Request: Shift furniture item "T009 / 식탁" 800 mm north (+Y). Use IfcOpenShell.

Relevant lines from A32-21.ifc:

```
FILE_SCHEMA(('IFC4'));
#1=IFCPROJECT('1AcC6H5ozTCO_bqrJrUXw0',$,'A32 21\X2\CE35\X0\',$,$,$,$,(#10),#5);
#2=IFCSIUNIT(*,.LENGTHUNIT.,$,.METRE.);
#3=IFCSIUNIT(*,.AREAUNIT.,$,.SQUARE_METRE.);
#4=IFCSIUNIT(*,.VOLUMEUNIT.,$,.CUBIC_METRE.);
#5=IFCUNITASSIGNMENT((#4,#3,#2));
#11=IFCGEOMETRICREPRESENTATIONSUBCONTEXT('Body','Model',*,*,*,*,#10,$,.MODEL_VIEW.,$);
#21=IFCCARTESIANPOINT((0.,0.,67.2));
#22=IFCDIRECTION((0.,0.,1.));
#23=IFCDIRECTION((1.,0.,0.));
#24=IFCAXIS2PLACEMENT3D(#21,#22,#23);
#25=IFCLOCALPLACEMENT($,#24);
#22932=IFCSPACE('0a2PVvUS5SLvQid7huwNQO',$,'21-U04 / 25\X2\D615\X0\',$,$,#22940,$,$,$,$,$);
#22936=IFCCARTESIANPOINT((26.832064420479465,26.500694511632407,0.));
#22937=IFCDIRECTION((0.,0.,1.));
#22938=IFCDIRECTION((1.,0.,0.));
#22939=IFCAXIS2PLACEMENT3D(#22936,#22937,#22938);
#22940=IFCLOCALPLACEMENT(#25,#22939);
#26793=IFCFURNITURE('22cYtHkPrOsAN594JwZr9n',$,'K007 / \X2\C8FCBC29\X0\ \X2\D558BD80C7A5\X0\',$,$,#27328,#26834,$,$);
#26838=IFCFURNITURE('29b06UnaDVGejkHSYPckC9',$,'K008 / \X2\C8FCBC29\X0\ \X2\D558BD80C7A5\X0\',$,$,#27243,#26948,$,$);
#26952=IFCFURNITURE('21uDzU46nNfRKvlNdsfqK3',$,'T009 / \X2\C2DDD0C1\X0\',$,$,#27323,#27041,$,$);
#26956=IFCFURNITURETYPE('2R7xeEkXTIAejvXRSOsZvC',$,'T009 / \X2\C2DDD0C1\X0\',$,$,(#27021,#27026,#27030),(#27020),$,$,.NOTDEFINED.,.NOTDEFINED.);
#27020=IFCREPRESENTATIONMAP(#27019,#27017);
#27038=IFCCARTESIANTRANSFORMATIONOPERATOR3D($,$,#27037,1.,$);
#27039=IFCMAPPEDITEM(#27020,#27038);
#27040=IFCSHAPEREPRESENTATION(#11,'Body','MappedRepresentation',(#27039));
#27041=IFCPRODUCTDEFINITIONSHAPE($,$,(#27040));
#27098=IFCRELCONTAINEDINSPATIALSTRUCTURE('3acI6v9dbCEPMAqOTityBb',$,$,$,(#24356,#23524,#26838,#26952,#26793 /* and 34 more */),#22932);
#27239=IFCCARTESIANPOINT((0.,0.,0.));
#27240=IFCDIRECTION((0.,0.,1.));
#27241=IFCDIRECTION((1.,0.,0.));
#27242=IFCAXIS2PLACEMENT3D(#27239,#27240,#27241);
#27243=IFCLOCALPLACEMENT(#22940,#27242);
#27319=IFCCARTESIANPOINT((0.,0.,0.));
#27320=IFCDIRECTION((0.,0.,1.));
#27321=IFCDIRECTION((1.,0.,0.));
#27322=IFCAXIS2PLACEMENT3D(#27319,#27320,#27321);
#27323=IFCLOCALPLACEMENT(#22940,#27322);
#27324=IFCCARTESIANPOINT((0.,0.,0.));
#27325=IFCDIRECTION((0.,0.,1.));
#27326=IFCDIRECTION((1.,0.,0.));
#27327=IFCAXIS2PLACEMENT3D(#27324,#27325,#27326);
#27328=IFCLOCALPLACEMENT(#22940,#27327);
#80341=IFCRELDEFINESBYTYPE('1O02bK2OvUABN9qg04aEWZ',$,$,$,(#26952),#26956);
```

```python
import ifcopenshell
import ifcopenshell.api.geometry
import ifcopenshell.util.placement

model = ifcopenshell.open("A32-21.ifc")

item = model.by_id(26952)
matrix = ifcopenshell.util.placement.get_local_placement(item.ObjectPlacement)
matrix[1, 3] += 0.8
ifcopenshell.api.geometry.edit_object_placement(model, product=item, matrix=matrix, is_si=False)

print(ifcopenshell.util.placement.get_local_placement(item.ObjectPlacement).round(3) + 0.0)

model.write("A32-21_updated.ifc")
```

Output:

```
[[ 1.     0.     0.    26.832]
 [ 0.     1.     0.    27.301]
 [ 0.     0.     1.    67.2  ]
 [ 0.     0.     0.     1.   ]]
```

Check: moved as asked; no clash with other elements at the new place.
